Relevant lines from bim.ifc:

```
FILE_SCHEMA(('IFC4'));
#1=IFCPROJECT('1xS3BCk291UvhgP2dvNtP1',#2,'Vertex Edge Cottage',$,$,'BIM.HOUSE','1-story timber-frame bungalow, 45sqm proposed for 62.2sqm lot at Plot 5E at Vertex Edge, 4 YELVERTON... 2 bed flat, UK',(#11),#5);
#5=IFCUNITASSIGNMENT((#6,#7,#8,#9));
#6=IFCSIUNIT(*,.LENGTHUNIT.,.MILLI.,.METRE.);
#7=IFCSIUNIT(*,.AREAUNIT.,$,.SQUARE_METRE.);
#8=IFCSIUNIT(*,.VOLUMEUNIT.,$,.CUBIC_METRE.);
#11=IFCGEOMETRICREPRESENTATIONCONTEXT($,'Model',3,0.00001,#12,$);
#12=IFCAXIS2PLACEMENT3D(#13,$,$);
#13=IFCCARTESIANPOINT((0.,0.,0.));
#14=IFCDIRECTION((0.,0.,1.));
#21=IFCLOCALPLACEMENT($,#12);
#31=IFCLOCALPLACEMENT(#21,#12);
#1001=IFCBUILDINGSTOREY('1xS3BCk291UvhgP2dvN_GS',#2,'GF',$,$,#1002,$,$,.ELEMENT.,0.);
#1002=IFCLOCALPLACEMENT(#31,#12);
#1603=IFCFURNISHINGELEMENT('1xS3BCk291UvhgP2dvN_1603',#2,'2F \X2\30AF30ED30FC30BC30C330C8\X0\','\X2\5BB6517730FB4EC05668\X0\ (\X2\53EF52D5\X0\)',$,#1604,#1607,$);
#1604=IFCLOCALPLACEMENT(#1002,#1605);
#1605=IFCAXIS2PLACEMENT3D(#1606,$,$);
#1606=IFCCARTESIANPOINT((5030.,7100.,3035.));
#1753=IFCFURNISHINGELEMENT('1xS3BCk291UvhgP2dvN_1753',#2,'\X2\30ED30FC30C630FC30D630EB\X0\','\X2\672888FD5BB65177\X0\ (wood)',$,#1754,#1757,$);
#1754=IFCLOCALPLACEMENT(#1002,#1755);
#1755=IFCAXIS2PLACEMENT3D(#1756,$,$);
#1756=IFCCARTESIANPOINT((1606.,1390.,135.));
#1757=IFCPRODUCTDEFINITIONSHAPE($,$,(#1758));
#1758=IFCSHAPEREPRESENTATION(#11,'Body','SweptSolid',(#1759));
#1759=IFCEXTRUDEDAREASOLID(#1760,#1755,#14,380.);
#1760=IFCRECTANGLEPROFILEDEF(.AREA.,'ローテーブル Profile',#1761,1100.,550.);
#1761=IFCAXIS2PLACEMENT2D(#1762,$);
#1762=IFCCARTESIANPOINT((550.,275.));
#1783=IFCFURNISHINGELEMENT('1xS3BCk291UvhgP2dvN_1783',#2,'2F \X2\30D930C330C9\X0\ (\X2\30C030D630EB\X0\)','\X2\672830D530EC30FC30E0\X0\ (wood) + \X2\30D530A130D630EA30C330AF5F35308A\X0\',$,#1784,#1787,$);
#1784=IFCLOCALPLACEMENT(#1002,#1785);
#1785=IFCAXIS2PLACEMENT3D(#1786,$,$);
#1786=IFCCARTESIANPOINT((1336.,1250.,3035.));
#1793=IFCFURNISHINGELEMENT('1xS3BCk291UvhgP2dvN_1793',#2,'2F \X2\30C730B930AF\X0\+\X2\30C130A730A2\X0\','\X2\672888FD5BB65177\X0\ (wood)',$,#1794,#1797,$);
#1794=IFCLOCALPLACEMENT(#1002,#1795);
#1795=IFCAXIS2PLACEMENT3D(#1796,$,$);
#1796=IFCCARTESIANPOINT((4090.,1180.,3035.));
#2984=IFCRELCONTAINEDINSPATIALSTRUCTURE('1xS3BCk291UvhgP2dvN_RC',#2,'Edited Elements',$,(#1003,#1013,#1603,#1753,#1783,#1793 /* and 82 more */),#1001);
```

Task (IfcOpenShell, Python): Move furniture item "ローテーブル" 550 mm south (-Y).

```python
import ifcopenshell
import ifcopenshell.api.geometry
import ifcopenshell.util.placement
import ifcopenshell.util.unit

model = ifcopenshell.open("bim.ifc")
unit_scale = ifcopenshell.util.unit.calculate_unit_scale(model)

item = model.by_guid("1xS3BCk291UvhgP2dvN_1753")
matrix = ifcopenshell.util.placement.get_local_placement(item.ObjectPlacement)
matrix[1, 3] -= 0.55 / unit_scale
ifcopenshell.api.geometry.edit_object_placement(model, product=item, matrix=matrix, is_si=False)

print(ifcopenshell.util.placement.get_local_placement(item.ObjectPlacement).round(3) + 0.0)

model.write("bim_edited.ifc")
```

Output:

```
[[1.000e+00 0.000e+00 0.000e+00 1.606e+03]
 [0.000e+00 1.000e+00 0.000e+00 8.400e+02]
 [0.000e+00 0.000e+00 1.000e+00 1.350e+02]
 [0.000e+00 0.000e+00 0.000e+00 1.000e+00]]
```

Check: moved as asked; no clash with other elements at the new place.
